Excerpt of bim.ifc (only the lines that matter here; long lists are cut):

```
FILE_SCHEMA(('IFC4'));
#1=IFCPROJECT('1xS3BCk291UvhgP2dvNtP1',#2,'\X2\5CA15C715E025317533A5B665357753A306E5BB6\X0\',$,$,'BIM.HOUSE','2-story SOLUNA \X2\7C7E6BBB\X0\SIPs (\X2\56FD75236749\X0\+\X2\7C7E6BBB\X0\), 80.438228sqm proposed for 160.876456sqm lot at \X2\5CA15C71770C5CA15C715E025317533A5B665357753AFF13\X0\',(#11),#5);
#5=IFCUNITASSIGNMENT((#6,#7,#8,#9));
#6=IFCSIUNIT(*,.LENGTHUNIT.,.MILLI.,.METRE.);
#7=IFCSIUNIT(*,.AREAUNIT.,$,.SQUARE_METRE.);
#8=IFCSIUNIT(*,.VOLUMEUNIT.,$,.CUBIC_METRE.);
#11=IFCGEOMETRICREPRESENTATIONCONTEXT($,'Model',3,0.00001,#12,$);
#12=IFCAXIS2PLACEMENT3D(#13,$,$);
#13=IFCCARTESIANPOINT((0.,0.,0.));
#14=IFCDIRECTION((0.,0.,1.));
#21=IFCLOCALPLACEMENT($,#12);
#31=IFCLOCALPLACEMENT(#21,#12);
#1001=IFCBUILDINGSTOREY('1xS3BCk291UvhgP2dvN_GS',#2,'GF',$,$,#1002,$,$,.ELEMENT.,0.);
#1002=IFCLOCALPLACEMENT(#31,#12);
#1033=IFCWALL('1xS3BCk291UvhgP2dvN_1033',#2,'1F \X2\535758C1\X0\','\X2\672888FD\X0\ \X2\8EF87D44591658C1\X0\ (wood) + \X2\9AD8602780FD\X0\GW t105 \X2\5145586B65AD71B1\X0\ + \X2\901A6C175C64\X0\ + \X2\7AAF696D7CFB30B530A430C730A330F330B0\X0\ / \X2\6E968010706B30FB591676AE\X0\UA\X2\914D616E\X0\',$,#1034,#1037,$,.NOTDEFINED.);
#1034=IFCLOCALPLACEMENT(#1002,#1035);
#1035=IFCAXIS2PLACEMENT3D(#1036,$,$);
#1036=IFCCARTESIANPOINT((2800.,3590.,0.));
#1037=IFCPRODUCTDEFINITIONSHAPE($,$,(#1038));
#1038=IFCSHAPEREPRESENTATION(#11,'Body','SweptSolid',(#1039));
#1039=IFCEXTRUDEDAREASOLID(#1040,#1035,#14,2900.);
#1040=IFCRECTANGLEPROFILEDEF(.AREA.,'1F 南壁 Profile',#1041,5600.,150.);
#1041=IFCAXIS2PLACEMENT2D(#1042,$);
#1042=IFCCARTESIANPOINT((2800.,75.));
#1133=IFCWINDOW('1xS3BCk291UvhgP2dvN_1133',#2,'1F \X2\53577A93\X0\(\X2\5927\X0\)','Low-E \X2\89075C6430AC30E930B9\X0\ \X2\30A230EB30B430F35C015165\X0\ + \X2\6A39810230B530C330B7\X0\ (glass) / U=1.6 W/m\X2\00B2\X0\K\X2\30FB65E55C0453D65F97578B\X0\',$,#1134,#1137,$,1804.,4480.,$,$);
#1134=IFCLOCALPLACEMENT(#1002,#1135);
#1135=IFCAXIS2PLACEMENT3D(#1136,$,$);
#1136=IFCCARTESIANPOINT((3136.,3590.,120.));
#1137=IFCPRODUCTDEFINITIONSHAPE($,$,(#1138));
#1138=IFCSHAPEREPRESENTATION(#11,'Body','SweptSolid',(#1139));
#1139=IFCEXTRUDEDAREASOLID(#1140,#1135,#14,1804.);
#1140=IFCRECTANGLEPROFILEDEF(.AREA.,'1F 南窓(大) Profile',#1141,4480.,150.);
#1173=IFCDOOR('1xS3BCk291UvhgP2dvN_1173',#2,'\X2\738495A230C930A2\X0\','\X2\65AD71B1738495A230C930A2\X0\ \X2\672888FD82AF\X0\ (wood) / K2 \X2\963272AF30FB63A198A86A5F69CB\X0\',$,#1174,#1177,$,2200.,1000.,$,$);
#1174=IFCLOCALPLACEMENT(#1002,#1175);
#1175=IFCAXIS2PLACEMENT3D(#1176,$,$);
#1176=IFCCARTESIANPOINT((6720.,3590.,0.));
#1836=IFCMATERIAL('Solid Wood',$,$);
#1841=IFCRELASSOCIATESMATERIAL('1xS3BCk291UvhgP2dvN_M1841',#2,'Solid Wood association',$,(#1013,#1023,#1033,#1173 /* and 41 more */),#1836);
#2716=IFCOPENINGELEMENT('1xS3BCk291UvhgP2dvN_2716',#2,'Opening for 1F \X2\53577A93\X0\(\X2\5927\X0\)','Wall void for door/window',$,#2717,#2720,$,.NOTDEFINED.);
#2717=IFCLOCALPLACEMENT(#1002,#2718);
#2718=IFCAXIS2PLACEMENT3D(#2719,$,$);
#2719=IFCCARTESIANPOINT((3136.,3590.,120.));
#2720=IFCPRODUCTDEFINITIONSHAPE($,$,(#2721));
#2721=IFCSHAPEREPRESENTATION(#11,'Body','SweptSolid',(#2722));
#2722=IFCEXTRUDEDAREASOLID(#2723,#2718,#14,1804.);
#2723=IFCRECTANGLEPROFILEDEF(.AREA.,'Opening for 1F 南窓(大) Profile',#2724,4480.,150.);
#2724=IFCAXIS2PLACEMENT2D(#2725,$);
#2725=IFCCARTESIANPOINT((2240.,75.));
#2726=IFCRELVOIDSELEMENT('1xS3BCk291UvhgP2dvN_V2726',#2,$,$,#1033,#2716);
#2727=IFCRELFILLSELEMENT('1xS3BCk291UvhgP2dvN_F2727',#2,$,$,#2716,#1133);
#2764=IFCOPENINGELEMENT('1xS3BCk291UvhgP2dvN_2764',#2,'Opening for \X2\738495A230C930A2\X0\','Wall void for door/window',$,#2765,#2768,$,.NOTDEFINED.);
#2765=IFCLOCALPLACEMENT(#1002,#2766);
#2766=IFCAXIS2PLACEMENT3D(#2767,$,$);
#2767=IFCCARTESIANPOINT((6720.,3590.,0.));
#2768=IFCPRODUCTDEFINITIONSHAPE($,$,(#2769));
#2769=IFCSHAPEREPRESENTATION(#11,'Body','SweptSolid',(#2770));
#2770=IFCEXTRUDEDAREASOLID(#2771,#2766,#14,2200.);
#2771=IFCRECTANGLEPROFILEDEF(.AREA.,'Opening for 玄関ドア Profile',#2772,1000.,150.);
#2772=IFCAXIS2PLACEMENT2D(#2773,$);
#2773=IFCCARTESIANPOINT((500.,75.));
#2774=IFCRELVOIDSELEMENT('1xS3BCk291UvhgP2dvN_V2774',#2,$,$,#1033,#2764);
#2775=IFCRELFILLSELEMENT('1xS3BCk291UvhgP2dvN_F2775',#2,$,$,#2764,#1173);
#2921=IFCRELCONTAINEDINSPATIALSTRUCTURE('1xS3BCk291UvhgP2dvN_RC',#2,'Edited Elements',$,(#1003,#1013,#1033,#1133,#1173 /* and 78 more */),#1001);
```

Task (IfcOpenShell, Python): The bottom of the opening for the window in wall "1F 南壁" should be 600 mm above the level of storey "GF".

```python
import numpy as np
import ifcopenshell
import ifcopenshell.api.geometry
import ifcopenshell.geom
import ifcopenshell.util.element
import ifcopenshell.util.placement
import ifcopenshell.util.shape
import ifcopenshell.util.unit

model = ifcopenshell.open("bim.ifc")
unit_scale = ifcopenshell.util.unit.calculate_unit_scale(model)

window = model.by_id(1133)
opening = window.FillsVoids[0].RelatingOpeningElement
storey = ifcopenshell.util.element.get_container(window, ifc_class="IfcBuildingStorey")
level = ifcopenshell.util.placement.get_local_placement(storey.ObjectPlacement)[2, 3]

# The opening's origin need not be at the sill, so measure its lowest point.
shape = ifcopenshell.geom.create_shape(ifcopenshell.geom.settings(), opening)
bottom = ifcopenshell.util.shape.get_shape_bottom_elevation(shape, shape.geometry) / unit_scale
dz = level + 0.6 / unit_scale - bottom

shift = np.array([0.0, 0.0, dz])
# The window is not placed relative to its opening, so move both.
for product in (opening, window):
    matrix = ifcopenshell.util.placement.get_local_placement(product.ObjectPlacement)
    matrix[:3, 3] += shift
    ifcopenshell.api.geometry.edit_object_placement(model, product=product, matrix=matrix, is_si=False)

print(f"moved by {dz * unit_scale:+.3f} m")

model.write("bim_updated.ifc")
```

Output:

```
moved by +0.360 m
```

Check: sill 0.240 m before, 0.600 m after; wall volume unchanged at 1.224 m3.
